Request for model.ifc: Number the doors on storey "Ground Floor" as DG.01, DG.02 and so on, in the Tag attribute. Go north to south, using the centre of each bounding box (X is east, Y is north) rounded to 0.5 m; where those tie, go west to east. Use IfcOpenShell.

First a look at what the model holds.

```python
import ifcopenshell
import ifcopenshell.util.element
import ifcopenshell.util.placement

model = ifcopenshell.open("model.ifc")
print(model.schema)
storey = next(s for s in model.by_type("IfcBuildingStorey") if s.Name == "Ground Floor")
doors = [e for e in ifcopenshell.util.element.get_decomposition(storey) if e.is_a("IfcDoor")]
for e in sorted(doors, key=lambda e: e.id()):
    origin = ifcopenshell.util.placement.get_local_placement(e.ObjectPlacement)[:3, 3]
    print(e.id(), e.Tag, e.Name, origin.round(2) + 0.0, sep=" | ")
```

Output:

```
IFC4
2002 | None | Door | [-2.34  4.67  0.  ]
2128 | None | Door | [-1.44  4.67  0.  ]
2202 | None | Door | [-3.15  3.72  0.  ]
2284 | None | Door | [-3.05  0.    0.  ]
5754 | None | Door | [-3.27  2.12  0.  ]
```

```python
import ifcopenshell
import ifcopenshell.geom
import ifcopenshell.util.element
import ifcopenshell.util.shape

model = ifcopenshell.open("model.ifc")
settings = ifcopenshell.geom.settings()
settings.set("use-world-coords", True)


def centre(element):
    shape = ifcopenshell.geom.create_shape(settings, element)
    return ifcopenshell.util.shape.get_bbox_centroid(shape.geometry)


storey = next(s for s in model.by_type("IfcBuildingStorey") if s.Name == "Ground Floor")
doors = [e for e in ifcopenshell.util.element.get_decomposition(storey) if e.is_a("IfcDoor")]

# Insertion points can sit at a corner or the storey origin, so sort by the geometry (in metres).
centres = {e: centre(e) for e in doors}
doors.sort(key=lambda e: (-round(centres[e][1] / 0.5), centres[e][0]))

for i, e in enumerate(doors, start=1):
    number = f"DG.{i:02d}"
    e.Tag = number
    print(e.id(), number)

model.write("model_edited.ifc")
```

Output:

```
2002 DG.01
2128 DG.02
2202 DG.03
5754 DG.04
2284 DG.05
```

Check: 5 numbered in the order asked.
